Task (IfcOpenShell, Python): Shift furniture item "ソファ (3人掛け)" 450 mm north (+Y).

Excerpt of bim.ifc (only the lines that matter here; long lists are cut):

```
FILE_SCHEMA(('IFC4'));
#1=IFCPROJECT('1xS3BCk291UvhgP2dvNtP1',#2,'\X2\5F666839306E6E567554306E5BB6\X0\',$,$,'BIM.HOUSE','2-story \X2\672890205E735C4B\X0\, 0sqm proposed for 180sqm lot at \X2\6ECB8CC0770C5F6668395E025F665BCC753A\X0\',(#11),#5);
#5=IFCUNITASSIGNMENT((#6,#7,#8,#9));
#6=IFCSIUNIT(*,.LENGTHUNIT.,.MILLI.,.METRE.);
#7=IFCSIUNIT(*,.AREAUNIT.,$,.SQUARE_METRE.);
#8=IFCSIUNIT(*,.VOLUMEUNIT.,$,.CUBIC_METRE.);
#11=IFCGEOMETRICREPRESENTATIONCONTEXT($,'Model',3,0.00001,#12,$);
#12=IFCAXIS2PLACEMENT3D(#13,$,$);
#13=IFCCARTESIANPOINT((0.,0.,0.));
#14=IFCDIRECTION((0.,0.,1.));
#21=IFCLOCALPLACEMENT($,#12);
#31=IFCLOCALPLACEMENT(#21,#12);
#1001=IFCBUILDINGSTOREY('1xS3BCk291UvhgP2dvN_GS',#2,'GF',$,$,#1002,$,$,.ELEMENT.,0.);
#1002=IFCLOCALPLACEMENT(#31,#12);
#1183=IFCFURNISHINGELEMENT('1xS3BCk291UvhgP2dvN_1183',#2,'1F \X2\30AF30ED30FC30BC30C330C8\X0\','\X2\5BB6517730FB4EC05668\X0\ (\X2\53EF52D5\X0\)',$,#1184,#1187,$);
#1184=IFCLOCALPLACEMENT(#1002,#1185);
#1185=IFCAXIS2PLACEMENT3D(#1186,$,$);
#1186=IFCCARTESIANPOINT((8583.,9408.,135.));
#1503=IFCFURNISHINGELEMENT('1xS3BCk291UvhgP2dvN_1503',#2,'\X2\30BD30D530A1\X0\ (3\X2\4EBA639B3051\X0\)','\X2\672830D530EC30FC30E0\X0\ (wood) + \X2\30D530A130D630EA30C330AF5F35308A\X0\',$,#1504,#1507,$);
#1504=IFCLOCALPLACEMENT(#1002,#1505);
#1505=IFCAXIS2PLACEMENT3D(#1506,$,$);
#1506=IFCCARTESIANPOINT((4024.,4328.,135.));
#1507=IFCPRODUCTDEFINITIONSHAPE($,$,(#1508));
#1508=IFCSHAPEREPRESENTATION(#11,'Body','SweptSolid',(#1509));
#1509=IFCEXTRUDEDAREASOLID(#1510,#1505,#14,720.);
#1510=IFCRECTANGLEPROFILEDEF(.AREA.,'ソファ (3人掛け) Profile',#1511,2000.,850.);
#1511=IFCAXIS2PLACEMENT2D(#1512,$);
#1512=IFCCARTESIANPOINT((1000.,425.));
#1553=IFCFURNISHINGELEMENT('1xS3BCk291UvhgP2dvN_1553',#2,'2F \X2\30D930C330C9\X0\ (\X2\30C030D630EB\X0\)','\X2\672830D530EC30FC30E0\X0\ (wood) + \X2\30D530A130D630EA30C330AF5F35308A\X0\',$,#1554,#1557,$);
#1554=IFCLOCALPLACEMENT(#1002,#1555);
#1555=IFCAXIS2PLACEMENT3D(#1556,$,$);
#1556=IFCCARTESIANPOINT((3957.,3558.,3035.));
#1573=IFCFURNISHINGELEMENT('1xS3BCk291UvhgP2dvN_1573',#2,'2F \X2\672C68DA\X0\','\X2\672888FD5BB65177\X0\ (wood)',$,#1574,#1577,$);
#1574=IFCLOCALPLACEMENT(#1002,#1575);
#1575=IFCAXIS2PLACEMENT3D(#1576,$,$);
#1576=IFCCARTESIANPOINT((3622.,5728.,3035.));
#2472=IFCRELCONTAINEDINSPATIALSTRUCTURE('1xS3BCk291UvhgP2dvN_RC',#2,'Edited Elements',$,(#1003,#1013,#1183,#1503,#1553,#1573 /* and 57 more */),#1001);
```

```python
import ifcopenshell
import ifcopenshell.api.geometry
import ifcopenshell.util.placement
import ifcopenshell.util.unit

model = ifcopenshell.open("bim.ifc")
unit_scale = ifcopenshell.util.unit.calculate_unit_scale(model)

item = model.by_guid("1xS3BCk291UvhgP2dvN_1503")
matrix = ifcopenshell.util.placement.get_local_placement(item.ObjectPlacement)
matrix[1, 3] += 0.45 / unit_scale
ifcopenshell.api.geometry.edit_object_placement(model, product=item, matrix=matrix, is_si=False)

print(ifcopenshell.util.placement.get_local_placement(item.ObjectPlacement).round(3) + 0.0)

model.write("bim_v2.ifc")
```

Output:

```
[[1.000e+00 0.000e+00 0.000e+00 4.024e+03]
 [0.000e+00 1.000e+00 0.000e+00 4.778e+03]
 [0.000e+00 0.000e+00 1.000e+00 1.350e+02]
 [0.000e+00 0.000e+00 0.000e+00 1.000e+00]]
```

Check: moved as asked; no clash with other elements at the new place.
